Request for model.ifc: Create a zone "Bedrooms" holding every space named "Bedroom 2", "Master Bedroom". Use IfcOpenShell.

First a look at what the model holds.

```python
import ifcopenshell

model = ifcopenshell.open("model.ifc")
print(model.schema)
seen = {}
for space in model.by_type("IfcSpace"):
    seen[space.LongName] = seen.get(space.LongName, 0) + 1
for name, count in sorted(seen.items(), key=str):
    print(count, "x", name)
print("zones:", [z.Name for z in model.by_type("IfcZone")][:20])
```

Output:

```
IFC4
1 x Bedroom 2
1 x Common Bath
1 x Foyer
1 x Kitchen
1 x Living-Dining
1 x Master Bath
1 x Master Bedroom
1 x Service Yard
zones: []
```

```python
import ifcopenshell
import ifcopenshell.api.group
import ifcopenshell.api.root

model = ifcopenshell.open("model.ifc")

names = {"Bedroom 2", "Master Bedroom"}
spaces = [s for s in model.by_type("IfcSpace") if s.LongName in names]

zone = ifcopenshell.api.root.create_entity(model, ifc_class="IfcZone", name="Bedrooms")
ifcopenshell.api.group.assign_group(model, products=spaces, group=zone)
print(len(spaces), "spaces in", zone.Name)

model.write("model-out.ifc")
```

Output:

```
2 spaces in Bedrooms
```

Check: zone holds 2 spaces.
